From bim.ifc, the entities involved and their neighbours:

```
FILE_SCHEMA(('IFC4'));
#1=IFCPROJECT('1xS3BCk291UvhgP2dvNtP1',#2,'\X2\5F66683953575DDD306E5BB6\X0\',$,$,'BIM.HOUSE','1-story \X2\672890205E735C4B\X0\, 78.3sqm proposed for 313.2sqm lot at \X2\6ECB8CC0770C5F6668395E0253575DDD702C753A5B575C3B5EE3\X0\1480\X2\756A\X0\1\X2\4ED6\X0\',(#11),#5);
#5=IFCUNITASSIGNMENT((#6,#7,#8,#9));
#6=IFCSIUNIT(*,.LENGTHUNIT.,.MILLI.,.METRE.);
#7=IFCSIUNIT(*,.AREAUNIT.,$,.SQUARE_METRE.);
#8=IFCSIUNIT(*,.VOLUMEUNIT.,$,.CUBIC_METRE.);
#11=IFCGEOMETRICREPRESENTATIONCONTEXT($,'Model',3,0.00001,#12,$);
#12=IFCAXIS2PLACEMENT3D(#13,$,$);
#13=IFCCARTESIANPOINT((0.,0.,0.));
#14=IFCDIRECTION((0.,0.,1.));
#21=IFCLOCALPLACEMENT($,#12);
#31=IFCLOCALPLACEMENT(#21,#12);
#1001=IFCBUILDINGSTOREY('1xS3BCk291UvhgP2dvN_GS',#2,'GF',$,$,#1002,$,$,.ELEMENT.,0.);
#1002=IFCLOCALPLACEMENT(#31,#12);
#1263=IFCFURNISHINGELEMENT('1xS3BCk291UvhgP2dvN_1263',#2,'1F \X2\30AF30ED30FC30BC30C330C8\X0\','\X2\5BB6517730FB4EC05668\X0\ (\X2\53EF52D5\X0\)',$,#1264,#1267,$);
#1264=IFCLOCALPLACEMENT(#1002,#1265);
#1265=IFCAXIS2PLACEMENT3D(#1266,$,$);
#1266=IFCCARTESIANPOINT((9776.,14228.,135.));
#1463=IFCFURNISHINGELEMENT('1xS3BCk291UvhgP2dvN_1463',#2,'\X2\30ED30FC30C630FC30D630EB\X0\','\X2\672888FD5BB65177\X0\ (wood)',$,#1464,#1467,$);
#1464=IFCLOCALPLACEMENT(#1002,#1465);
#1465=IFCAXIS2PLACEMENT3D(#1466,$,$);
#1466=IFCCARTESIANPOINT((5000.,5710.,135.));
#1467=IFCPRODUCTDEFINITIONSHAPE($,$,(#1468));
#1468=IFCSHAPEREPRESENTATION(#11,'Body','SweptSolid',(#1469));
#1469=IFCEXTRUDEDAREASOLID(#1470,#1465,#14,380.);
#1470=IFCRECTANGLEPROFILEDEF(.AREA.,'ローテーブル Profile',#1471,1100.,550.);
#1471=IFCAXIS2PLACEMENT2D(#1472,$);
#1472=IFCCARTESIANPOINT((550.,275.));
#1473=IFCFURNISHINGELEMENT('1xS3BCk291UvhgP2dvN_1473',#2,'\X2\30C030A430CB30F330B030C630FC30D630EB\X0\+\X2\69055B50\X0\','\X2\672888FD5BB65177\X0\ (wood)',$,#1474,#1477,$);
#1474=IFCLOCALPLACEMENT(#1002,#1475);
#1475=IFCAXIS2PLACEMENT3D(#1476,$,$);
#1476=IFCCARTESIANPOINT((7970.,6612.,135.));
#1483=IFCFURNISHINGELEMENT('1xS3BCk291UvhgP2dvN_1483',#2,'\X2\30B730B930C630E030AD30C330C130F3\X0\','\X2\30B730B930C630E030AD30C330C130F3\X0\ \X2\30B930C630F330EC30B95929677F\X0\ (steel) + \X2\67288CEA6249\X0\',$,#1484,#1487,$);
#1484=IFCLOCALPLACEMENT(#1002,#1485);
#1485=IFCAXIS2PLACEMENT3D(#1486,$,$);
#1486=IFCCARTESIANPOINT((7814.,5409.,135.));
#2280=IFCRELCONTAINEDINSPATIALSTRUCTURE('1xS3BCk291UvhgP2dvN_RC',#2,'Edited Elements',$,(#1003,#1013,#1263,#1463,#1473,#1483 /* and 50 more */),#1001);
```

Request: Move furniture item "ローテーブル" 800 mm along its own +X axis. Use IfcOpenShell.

```python
import ifcopenshell
import ifcopenshell.api.geometry
import ifcopenshell.util.placement

model = ifcopenshell.open("bim.ifc")

item = model.by_guid("1xS3BCk291UvhgP2dvN_1463")
matrix = ifcopenshell.util.placement.get_local_placement(item.ObjectPlacement)
matrix[:3, 3] += matrix[:3, 0] * 800.0
ifcopenshell.api.geometry.edit_object_placement(model, product=item, matrix=matrix, is_si=False)

print(ifcopenshell.util.placement.get_local_placement(item.ObjectPlacement).round(3) + 0.0)

model.write("bim_rev.ifc")
```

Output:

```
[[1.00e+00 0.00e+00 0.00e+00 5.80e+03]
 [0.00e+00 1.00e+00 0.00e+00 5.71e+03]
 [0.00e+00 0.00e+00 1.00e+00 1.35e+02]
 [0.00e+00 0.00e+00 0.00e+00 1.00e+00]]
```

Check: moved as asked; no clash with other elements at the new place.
